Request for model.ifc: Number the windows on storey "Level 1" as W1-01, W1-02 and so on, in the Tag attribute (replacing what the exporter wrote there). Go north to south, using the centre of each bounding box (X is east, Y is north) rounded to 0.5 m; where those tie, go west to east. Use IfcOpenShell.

First a look at what the model holds.

```python
import ifcopenshell
import ifcopenshell.util.element
import ifcopenshell.util.placement

model = ifcopenshell.open("model.ifc")
print(model.schema)
storey = next(s for s in model.by_type("IfcBuildingStorey") if s.Name == "Level 1")
windows = [e for e in ifcopenshell.util.element.get_decomposition(storey) if e.is_a("IfcWindow")]
for e in sorted(windows, key=lambda e: e.id()):
    origin = ifcopenshell.util.placement.get_local_placement(e.ObjectPlacement)[:3, 3]
    print(e.id(), e.Tag, e.Name, origin.round(2) + 0.0, sep=" | ")
```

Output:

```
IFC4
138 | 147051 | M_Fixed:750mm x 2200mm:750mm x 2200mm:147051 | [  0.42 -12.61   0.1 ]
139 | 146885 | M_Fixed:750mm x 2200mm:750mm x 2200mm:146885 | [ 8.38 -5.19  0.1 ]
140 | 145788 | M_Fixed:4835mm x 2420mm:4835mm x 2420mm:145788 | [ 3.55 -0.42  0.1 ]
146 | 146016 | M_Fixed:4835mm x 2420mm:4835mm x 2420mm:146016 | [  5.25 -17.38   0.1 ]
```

```python
import ifcopenshell
import ifcopenshell.geom
import ifcopenshell.util.element
import ifcopenshell.util.shape

model = ifcopenshell.open("model.ifc")
settings = ifcopenshell.geom.settings()
settings.set("use-world-coords", True)


def centre(element):
    shape = ifcopenshell.geom.create_shape(settings, element)
    return ifcopenshell.util.shape.get_bbox_centroid(shape.geometry)


storey = next(s for s in model.by_type("IfcBuildingStorey") if s.Name == "Level 1")
windows = [e for e in ifcopenshell.util.element.get_decomposition(storey) if e.is_a("IfcWindow")]

# Insertion points can sit at a corner or the storey origin, so sort by the geometry (in metres).
centres = {e: centre(e) for e in windows}
windows.sort(key=lambda e: (-round(centres[e][1] / 0.5), centres[e][0]))

for i, e in enumerate(windows, start=1):
    number = f"W1-{i:02d}"
    e.Tag = number
    print(e.id(), number)

model.write("model_edited.ifc")
```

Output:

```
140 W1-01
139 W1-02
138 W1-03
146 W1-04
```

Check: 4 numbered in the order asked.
